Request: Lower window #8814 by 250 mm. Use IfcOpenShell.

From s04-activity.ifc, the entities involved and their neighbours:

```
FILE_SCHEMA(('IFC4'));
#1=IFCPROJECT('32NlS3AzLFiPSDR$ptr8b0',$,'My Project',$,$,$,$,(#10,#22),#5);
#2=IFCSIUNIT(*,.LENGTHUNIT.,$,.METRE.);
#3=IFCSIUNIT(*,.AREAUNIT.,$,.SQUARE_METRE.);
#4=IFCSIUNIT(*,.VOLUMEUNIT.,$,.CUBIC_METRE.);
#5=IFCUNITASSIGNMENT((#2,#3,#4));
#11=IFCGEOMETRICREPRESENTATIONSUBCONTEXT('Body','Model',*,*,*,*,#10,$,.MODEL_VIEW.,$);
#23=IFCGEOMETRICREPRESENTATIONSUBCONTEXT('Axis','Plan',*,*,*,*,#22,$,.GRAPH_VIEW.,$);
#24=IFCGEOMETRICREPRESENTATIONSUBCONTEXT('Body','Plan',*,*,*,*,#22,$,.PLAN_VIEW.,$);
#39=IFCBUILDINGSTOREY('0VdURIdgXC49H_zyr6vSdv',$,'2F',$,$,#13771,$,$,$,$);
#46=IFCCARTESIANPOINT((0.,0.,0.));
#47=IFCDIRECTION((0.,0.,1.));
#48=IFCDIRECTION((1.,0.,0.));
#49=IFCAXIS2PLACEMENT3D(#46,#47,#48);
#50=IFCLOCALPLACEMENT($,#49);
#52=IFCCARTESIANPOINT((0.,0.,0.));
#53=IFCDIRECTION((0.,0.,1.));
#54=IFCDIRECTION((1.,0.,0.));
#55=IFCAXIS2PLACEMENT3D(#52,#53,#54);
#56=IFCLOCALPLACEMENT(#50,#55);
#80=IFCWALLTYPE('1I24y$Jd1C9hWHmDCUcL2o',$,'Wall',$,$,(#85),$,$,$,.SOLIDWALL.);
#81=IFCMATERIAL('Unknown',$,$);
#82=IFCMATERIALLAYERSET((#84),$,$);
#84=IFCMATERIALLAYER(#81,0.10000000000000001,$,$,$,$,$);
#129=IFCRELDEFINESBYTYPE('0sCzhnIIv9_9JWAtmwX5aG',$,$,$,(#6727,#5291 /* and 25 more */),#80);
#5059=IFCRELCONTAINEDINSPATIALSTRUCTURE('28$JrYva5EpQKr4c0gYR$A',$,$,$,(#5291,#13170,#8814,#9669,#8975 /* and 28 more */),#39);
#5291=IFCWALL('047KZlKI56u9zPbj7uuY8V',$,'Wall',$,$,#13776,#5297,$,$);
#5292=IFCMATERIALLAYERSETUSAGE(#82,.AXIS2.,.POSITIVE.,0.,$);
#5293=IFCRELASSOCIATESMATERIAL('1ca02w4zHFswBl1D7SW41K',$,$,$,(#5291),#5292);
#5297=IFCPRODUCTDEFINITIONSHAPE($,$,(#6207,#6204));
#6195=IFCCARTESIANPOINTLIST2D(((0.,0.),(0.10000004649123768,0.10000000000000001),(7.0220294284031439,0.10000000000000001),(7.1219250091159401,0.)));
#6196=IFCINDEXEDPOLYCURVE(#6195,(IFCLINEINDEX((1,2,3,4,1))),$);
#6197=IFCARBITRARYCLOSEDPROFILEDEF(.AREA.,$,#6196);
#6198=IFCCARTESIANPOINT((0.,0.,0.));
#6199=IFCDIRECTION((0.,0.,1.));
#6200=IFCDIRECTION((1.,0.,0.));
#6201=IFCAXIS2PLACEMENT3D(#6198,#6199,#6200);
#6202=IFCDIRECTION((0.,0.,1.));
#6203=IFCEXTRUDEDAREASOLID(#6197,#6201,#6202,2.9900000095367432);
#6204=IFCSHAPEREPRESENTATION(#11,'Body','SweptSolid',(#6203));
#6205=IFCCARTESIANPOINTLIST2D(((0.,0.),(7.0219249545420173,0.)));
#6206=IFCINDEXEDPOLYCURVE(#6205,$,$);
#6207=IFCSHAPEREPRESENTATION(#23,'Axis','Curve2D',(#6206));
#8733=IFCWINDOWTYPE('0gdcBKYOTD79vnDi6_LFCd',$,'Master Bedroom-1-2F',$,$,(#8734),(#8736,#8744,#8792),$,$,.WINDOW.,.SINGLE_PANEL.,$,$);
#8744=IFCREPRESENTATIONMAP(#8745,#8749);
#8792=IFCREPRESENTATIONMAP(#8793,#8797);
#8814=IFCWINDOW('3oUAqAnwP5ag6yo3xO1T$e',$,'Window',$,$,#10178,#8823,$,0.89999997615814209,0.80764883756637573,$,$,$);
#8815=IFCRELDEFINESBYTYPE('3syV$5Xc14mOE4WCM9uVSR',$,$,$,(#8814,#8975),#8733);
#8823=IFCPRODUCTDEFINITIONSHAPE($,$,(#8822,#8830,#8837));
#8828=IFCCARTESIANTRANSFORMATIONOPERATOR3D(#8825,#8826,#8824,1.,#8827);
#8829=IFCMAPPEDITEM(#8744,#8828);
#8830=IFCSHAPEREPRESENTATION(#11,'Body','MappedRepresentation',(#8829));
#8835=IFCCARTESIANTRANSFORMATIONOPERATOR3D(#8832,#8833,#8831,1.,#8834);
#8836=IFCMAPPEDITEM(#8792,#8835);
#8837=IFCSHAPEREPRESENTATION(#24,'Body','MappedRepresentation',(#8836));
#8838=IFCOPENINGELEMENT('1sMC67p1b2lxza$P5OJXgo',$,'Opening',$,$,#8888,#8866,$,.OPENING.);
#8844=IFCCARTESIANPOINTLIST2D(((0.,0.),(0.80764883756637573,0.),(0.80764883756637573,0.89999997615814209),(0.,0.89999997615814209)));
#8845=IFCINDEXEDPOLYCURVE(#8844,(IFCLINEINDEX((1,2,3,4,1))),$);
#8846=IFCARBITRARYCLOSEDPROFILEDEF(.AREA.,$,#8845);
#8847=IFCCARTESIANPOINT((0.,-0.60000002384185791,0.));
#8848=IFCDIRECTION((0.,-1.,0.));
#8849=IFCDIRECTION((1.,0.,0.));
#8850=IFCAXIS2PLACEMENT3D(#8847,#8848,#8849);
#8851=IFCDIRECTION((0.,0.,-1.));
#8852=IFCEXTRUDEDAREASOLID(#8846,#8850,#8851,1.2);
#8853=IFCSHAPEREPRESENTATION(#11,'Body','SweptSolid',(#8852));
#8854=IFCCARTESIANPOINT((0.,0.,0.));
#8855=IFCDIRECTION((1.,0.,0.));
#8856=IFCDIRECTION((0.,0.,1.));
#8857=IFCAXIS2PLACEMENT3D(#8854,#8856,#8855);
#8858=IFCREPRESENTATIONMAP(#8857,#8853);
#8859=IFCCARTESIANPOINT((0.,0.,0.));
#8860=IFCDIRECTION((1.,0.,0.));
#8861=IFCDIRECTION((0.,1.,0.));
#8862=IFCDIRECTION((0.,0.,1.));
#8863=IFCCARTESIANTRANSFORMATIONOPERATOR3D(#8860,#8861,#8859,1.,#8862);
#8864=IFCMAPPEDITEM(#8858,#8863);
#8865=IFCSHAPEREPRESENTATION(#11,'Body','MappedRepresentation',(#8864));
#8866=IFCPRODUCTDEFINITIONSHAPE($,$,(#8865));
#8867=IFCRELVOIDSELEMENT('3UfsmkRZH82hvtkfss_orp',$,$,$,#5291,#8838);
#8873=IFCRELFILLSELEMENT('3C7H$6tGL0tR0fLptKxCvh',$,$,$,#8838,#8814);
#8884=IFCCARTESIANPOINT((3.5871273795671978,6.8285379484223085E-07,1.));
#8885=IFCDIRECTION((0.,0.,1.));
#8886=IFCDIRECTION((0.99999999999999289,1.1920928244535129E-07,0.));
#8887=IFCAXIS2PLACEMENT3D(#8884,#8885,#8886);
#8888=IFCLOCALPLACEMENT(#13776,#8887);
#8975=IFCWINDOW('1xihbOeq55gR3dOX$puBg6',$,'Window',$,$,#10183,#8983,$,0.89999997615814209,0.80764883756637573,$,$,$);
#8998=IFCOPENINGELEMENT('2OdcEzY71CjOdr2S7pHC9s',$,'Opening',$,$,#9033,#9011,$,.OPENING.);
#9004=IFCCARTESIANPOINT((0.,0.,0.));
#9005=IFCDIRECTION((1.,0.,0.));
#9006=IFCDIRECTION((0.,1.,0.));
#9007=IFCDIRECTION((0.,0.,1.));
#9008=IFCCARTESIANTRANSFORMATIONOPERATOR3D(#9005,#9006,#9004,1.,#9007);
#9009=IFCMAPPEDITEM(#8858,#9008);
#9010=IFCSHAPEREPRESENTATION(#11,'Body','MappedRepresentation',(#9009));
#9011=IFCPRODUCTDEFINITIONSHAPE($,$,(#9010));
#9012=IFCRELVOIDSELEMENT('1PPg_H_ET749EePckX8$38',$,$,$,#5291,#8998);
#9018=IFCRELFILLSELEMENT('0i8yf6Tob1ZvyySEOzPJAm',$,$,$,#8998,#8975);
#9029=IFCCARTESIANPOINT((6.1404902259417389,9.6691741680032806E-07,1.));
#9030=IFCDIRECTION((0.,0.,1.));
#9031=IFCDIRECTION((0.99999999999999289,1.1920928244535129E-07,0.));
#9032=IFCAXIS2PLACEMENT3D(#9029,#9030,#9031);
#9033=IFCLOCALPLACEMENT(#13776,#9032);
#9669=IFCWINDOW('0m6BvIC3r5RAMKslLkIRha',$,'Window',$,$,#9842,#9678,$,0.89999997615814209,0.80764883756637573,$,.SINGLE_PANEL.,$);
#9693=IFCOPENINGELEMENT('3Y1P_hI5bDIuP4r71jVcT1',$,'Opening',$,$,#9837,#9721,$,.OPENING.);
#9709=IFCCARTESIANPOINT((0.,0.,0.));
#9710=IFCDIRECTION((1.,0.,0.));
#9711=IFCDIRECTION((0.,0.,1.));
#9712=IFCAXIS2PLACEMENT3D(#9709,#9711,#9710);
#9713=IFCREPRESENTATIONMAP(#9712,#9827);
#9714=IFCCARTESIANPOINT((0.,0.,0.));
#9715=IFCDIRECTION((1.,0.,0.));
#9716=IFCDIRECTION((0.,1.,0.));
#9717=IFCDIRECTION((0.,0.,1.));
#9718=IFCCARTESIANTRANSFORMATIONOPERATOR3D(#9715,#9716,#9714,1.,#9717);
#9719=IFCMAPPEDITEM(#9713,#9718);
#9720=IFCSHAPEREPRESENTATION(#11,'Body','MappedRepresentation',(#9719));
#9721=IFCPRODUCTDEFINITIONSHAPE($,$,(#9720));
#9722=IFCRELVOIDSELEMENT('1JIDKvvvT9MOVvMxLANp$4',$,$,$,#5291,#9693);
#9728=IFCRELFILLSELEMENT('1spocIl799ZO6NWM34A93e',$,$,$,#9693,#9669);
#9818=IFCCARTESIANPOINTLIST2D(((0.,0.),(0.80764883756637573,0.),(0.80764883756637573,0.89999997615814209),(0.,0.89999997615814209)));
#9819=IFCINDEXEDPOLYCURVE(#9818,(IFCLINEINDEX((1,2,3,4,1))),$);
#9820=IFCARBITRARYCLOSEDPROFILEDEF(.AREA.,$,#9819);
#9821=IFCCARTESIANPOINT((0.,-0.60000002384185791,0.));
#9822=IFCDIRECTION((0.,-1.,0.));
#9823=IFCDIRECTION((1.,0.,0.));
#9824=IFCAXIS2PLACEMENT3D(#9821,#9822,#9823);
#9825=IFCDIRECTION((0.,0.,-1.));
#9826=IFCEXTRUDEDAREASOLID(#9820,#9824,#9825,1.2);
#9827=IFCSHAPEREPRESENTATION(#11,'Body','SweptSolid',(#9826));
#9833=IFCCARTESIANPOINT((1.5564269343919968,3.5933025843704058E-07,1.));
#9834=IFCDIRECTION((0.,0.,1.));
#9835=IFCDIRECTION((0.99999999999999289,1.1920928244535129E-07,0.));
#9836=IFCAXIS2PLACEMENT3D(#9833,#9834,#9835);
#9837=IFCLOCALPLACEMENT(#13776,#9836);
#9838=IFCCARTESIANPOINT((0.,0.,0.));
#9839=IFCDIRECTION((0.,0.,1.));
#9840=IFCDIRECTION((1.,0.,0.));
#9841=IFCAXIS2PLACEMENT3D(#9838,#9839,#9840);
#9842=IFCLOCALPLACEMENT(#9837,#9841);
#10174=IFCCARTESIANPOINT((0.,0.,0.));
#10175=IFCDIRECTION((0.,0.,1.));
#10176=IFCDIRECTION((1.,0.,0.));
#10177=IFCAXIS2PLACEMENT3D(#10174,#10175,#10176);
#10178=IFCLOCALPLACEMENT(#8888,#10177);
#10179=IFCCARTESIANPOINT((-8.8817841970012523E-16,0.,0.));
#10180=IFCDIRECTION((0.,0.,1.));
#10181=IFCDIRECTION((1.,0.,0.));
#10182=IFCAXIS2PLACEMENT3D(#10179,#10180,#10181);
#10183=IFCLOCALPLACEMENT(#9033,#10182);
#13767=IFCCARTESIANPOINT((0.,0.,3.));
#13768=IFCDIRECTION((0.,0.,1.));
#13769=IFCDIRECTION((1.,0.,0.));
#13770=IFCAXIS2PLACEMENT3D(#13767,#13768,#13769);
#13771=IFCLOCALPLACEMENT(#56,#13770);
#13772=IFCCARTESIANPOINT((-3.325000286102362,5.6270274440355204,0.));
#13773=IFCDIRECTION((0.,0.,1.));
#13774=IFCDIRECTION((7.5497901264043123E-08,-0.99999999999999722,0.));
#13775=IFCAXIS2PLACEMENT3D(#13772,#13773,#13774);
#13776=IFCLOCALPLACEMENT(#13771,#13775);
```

```python
import numpy as np
import ifcopenshell
import ifcopenshell.api.geometry
import ifcopenshell.util.placement
import ifcopenshell.util.unit

model = ifcopenshell.open("s04-activity.ifc")
unit_scale = ifcopenshell.util.unit.calculate_unit_scale(model)

window = model.by_guid("3oUAqAnwP5ag6yo3xO1T$e")
opening = window.FillsVoids[0].RelatingOpeningElement
dz = -0.25

shift = np.array([0.0, 0.0, dz])
# The window is placed relative to its opening, so it follows when the opening moves.
matrix = ifcopenshell.util.placement.get_local_placement(opening.ObjectPlacement)
matrix[:3, 3] += shift
ifcopenshell.api.geometry.edit_object_placement(
    model, product=opening, matrix=matrix, is_si=False, should_transform_children=True
)

print(f"moved by {dz * unit_scale:+.3f} m")

model.write("s04-activity_rev.ifc")
```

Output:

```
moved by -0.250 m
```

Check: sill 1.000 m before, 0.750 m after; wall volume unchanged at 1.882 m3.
